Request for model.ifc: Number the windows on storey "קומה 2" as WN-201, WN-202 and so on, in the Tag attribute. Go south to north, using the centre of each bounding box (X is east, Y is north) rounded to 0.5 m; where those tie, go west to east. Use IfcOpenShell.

First a look at what the model holds.

```python
import ifcopenshell
import ifcopenshell.util.element
import ifcopenshell.util.placement

model = ifcopenshell.open("model.ifc")
print(model.schema)
storey = next(s for s in model.by_type("IfcBuildingStorey") if s.Name == "קומה 2")
windows = [e for e in ifcopenshell.util.element.get_decomposition(storey) if e.is_a("IfcWindow")]
for e in sorted(windows, key=lambda e: e.id()):
    origin = ifcopenshell.util.placement.get_local_placement(e.ObjectPlacement)[:3, 3]
    print(e.id(), e.Tag, e.Name, origin.round(2) + 0.0, sep=" | ")
```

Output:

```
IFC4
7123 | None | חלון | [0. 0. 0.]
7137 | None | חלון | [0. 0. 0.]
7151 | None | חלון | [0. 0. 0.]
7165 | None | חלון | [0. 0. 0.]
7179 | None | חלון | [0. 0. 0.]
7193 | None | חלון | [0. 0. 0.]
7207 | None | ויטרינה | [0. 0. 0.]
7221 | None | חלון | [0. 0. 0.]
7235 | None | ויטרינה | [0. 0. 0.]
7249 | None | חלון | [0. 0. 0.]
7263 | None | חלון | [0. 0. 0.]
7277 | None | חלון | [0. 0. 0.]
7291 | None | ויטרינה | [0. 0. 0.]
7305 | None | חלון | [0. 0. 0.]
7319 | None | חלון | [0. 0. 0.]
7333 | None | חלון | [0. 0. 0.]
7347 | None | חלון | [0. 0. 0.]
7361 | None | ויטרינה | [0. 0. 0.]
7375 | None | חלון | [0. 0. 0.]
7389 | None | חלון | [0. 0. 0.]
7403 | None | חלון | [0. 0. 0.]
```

```python
import ifcopenshell
import ifcopenshell.geom
import ifcopenshell.util.element
import ifcopenshell.util.shape

model = ifcopenshell.open("model.ifc")
settings = ifcopenshell.geom.settings()
settings.set("use-world-coords", True)


def centre(element):
    shape = ifcopenshell.geom.create_shape(settings, element)
    return ifcopenshell.util.shape.get_bbox_centroid(shape.geometry)


storey = next(s for s in model.by_type("IfcBuildingStorey") if s.Name == "קומה 2")
windows = [e for e in ifcopenshell.util.element.get_decomposition(storey) if e.is_a("IfcWindow")]

# Insertion points can sit at a corner or the storey origin, so sort by the geometry (in metres).
centres = {e: centre(e) for e in windows}
windows.sort(key=lambda e: (round(centres[e][1] / 0.5), centres[e][0]))

for i, e in enumerate(windows, start=1):
    number = f"WN-2{i:02d}"
    e.Tag = number
    print(e.id(), number)

model.write("model_rev.ifc")
```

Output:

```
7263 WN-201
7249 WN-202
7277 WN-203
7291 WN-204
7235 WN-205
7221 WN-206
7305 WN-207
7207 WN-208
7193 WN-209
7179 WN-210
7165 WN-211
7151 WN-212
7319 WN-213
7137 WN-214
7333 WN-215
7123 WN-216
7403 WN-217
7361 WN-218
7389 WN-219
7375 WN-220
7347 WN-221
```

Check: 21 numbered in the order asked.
